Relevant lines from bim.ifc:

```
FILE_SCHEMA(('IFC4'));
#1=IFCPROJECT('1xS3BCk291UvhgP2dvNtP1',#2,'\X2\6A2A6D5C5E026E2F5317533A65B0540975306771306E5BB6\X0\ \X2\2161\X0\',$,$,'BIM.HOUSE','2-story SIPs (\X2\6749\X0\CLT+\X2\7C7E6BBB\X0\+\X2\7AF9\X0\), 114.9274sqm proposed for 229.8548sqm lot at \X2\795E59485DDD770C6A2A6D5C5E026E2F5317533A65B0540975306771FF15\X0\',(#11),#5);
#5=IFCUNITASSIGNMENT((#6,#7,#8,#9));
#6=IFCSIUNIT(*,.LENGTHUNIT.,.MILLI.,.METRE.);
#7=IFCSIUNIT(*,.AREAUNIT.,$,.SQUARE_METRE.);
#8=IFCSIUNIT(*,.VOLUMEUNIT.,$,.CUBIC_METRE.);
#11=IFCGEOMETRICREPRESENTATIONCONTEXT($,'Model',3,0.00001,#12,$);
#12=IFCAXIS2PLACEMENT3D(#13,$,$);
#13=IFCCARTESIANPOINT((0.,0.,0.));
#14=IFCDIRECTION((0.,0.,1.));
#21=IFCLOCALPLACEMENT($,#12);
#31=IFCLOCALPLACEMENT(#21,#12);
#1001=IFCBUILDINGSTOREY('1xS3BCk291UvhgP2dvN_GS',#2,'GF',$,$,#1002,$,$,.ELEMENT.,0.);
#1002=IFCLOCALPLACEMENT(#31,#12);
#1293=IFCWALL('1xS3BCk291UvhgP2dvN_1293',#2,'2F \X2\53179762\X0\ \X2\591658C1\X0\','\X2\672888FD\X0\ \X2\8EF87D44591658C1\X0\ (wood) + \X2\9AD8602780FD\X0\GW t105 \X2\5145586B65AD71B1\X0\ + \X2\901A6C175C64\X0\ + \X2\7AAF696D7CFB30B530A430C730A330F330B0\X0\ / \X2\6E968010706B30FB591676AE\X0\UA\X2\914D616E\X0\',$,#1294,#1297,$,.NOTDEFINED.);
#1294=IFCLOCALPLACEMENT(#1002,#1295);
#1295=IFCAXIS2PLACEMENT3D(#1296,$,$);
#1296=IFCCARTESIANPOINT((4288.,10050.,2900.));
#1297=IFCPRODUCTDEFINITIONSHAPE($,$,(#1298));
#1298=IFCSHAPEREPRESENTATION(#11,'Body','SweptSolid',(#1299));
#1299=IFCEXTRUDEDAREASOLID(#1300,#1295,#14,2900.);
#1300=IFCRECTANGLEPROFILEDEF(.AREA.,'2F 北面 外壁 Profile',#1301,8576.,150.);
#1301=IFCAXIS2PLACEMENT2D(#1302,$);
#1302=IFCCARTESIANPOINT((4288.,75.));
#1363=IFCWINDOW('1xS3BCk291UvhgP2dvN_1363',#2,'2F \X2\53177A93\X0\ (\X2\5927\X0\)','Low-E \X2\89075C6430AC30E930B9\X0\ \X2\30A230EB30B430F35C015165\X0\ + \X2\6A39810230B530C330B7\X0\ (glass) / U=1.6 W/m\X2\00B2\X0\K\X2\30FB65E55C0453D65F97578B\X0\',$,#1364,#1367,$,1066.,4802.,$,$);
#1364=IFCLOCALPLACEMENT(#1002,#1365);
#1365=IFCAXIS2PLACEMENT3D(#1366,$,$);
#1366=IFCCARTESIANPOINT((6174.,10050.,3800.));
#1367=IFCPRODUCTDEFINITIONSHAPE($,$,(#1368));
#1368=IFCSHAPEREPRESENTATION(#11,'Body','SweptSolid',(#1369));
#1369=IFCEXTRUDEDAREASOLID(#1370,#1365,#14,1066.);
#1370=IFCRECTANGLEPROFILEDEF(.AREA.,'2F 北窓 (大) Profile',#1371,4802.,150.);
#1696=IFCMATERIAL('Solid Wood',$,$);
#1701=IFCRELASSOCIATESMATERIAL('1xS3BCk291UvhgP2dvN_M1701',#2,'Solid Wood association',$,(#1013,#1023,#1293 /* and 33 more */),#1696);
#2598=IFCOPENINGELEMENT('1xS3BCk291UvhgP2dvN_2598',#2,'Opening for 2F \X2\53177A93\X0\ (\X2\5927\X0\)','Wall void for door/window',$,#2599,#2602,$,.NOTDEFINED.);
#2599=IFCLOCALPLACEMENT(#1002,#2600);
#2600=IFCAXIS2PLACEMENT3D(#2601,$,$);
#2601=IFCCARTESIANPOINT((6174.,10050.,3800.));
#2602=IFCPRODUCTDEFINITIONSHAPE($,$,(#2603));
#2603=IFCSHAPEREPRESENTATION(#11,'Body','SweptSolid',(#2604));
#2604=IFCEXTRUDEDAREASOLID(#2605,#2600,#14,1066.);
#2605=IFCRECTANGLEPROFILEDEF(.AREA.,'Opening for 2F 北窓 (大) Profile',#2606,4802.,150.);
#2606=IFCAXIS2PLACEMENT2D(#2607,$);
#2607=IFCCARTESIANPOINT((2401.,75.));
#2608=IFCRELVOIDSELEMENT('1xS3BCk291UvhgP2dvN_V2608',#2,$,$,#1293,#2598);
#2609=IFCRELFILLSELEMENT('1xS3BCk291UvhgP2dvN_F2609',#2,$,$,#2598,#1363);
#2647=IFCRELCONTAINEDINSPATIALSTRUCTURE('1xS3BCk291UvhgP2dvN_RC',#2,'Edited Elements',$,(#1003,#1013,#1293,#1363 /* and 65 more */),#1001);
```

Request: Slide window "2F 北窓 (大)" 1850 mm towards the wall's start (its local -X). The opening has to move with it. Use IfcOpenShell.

```python
import ifcopenshell
import ifcopenshell.api.geometry
import ifcopenshell.util.placement
import ifcopenshell.util.unit

model = ifcopenshell.open("bim.ifc")
unit_scale = ifcopenshell.util.unit.calculate_unit_scale(model)

window = model.by_id(1363)
opening = window.FillsVoids[0].RelatingOpeningElement
wall = opening.VoidsElements[0].RelatingBuildingElement

wall_matrix = ifcopenshell.util.placement.get_local_placement(wall.ObjectPlacement)
shift = wall_matrix[:3, 0] * -1.85 / unit_scale
before = ifcopenshell.util.placement.get_local_placement(window.ObjectPlacement)[:3, 3].copy()

# The window is not placed relative to its opening, so move both.
for product in (opening, window):
    matrix = ifcopenshell.util.placement.get_local_placement(product.ObjectPlacement)
    matrix[:3, 3] += shift
    ifcopenshell.api.geometry.edit_object_placement(model, product=product, matrix=matrix, is_si=False)

after = ifcopenshell.util.placement.get_local_placement(window.ObjectPlacement)[:3, 3]
print("window moved by", (after - before).round(3) + 0.0)

model.write("bim-out.ifc")
```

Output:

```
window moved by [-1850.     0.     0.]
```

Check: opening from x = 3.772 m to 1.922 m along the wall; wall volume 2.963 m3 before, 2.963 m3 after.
